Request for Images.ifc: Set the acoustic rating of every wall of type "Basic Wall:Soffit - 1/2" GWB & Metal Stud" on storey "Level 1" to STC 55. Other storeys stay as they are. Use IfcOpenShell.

First a look at what the model holds.

```python
import ifcopenshell
import ifcopenshell.util.element

model = ifcopenshell.open("Images.ifc")
print(model.schema)
storey = next(s for s in model.by_type("IfcBuildingStorey") if s.Name == "Level 1")
walls = [e for e in ifcopenshell.util.element.get_decomposition(storey) if e.is_a("IfcWall")]
seen = {}
for e in walls:
    element_type = ifcopenshell.util.element.get_type(e)
    key = (element_type.Name if element_type != e and element_type else None, ifcopenshell.util.element.get_pset(e, "Pset_WallCommon", "AcousticRating"))
    seen[key] = seen.get(key, 0) + 1
for (name, value), count in sorted(seen.items(), key=str):
    print(count, "x", name, "|", value)
```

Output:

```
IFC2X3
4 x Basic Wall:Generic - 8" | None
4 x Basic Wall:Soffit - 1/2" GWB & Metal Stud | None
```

```python
import ifcopenshell
import ifcopenshell.api.pset
import ifcopenshell.util.element

model = ifcopenshell.open("Images.ifc")

storey = next(s for s in model.by_type("IfcBuildingStorey") if s.Name == "Level 1")
walls = [e for e in ifcopenshell.util.element.get_decomposition(storey) if e.is_a("IfcWall")]

count = 0
for e in walls:
    element_type = ifcopenshell.util.element.get_type(e)
    if element_type in (None, e) or element_type.Name != 'Basic Wall:Soffit - 1/2" GWB & Metal Stud':
        continue
    # add_pset returns the element's existing set when there is one.
    pset = ifcopenshell.api.pset.add_pset(model, product=e, name="Pset_WallCommon")
    ifcopenshell.api.pset.edit_pset(model, pset=pset, properties={"AcousticRating": "STC 55"})
    count += 1

print(count, "walls updated")

model.write("Images_rev.ifc")
```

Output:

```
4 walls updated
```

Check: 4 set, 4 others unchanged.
